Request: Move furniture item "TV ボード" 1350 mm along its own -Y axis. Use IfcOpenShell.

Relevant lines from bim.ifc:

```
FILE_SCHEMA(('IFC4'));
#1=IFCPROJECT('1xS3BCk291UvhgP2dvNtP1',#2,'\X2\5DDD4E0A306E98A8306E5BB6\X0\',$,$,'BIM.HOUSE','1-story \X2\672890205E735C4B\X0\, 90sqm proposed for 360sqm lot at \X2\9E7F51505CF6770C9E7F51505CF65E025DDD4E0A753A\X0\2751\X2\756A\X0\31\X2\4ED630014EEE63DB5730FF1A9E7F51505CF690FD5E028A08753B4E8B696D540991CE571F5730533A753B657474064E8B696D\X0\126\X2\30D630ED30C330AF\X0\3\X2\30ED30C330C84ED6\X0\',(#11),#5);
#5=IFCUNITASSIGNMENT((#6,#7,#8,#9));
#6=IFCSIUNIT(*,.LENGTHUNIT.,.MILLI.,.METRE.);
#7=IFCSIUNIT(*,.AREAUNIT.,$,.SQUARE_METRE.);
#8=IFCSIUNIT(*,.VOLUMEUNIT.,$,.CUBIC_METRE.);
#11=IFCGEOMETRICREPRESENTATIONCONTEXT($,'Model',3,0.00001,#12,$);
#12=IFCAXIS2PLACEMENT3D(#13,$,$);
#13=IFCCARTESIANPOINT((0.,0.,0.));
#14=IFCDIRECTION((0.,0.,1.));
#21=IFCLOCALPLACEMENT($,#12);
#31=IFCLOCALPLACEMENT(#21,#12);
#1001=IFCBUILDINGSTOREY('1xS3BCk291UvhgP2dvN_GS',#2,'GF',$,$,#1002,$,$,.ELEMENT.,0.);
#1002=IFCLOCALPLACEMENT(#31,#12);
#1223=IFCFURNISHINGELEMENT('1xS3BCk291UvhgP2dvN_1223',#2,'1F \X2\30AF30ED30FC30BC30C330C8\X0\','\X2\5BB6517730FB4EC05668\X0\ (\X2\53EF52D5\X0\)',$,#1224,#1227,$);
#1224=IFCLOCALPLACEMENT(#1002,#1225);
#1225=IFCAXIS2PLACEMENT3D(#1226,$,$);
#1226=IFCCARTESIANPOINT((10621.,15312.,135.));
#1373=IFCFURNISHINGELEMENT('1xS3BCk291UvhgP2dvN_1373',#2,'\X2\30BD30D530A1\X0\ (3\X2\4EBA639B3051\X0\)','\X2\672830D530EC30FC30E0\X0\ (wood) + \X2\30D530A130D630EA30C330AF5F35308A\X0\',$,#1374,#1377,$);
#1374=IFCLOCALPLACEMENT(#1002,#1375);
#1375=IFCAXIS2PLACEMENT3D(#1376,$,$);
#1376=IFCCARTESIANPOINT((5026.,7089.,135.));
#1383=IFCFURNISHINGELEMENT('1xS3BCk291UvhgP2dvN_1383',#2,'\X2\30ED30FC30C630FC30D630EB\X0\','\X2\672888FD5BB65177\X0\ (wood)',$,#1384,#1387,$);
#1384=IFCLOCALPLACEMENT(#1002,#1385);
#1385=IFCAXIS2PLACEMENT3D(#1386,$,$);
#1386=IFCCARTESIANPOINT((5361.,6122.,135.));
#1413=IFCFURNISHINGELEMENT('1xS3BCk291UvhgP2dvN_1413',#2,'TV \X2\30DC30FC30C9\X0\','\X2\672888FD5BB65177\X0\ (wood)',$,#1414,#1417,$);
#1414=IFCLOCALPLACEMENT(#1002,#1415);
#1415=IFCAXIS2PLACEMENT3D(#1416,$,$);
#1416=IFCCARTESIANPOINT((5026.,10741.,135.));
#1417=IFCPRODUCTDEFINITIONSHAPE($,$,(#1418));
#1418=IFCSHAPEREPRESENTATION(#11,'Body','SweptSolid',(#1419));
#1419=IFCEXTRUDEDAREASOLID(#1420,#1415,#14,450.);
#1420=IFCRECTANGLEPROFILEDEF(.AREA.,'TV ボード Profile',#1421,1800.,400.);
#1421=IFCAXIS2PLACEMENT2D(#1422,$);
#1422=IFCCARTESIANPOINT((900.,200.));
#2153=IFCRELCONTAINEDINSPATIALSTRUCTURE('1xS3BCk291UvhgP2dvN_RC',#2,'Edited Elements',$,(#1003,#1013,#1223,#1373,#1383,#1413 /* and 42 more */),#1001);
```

```python
import ifcopenshell
import ifcopenshell.api.geometry
import ifcopenshell.util.placement

model = ifcopenshell.open("bim.ifc")

item = model.by_guid("1xS3BCk291UvhgP2dvN_1413")
matrix = ifcopenshell.util.placement.get_local_placement(item.ObjectPlacement)
matrix[:3, 3] -= matrix[:3, 1] * 1350.0
ifcopenshell.api.geometry.edit_object_placement(model, product=item, matrix=matrix, is_si=False)

print(ifcopenshell.util.placement.get_local_placement(item.ObjectPlacement).round(3) + 0.0)

model.write("bim_updated.ifc")
```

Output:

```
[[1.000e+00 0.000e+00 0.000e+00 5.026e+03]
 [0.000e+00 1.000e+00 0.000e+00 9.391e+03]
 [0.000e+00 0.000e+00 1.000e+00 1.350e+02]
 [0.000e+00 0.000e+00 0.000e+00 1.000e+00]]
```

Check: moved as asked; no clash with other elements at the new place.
